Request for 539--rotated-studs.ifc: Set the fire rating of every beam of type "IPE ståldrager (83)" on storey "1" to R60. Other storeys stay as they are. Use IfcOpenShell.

First a look at what the model holds.

```python
import ifcopenshell
import ifcopenshell.util.element

model = ifcopenshell.open("539--rotated-studs.ifc")
print(model.schema)
storey = next(s for s in model.by_type("IfcBuildingStorey") if s.Name == "1")
beams = [e for e in ifcopenshell.util.element.get_decomposition(storey) if e.is_a("IfcBeam")]
seen = {}
for e in beams:
    element_type = ifcopenshell.util.element.get_type(e)
    key = (element_type.Name if element_type != e and element_type else None, ifcopenshell.util.element.get_pset(e, "Pset_BeamCommon", "FireRating"))
    seen[key] = seen.get(key, 0) + 1
for (name, value), count in sorted(seen.items(), key=str):
    print(count, "x", name, "|", value)
```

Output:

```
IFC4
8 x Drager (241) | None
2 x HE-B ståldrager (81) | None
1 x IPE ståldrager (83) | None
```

```python
import ifcopenshell
import ifcopenshell.api.pset
import ifcopenshell.util.element

model = ifcopenshell.open("539--rotated-studs.ifc")

storey = next(s for s in model.by_type("IfcBuildingStorey") if s.Name == "1")
beams = [e for e in ifcopenshell.util.element.get_decomposition(storey) if e.is_a("IfcBeam")]

count = 0
for e in beams:
    element_type = ifcopenshell.util.element.get_type(e)
    if element_type in (None, e) or element_type.Name != "IPE ståldrager (83)":
        continue
    # add_pset returns the element's existing set when there is one.
    pset = ifcopenshell.api.pset.add_pset(model, product=e, name="Pset_BeamCommon")
    ifcopenshell.api.pset.edit_pset(model, pset=pset, properties={"FireRating": "R60"})
    count += 1

print(count, "beams updated")

model.write("539--rotated-studs_rev.ifc")
```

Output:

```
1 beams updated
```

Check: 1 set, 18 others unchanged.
